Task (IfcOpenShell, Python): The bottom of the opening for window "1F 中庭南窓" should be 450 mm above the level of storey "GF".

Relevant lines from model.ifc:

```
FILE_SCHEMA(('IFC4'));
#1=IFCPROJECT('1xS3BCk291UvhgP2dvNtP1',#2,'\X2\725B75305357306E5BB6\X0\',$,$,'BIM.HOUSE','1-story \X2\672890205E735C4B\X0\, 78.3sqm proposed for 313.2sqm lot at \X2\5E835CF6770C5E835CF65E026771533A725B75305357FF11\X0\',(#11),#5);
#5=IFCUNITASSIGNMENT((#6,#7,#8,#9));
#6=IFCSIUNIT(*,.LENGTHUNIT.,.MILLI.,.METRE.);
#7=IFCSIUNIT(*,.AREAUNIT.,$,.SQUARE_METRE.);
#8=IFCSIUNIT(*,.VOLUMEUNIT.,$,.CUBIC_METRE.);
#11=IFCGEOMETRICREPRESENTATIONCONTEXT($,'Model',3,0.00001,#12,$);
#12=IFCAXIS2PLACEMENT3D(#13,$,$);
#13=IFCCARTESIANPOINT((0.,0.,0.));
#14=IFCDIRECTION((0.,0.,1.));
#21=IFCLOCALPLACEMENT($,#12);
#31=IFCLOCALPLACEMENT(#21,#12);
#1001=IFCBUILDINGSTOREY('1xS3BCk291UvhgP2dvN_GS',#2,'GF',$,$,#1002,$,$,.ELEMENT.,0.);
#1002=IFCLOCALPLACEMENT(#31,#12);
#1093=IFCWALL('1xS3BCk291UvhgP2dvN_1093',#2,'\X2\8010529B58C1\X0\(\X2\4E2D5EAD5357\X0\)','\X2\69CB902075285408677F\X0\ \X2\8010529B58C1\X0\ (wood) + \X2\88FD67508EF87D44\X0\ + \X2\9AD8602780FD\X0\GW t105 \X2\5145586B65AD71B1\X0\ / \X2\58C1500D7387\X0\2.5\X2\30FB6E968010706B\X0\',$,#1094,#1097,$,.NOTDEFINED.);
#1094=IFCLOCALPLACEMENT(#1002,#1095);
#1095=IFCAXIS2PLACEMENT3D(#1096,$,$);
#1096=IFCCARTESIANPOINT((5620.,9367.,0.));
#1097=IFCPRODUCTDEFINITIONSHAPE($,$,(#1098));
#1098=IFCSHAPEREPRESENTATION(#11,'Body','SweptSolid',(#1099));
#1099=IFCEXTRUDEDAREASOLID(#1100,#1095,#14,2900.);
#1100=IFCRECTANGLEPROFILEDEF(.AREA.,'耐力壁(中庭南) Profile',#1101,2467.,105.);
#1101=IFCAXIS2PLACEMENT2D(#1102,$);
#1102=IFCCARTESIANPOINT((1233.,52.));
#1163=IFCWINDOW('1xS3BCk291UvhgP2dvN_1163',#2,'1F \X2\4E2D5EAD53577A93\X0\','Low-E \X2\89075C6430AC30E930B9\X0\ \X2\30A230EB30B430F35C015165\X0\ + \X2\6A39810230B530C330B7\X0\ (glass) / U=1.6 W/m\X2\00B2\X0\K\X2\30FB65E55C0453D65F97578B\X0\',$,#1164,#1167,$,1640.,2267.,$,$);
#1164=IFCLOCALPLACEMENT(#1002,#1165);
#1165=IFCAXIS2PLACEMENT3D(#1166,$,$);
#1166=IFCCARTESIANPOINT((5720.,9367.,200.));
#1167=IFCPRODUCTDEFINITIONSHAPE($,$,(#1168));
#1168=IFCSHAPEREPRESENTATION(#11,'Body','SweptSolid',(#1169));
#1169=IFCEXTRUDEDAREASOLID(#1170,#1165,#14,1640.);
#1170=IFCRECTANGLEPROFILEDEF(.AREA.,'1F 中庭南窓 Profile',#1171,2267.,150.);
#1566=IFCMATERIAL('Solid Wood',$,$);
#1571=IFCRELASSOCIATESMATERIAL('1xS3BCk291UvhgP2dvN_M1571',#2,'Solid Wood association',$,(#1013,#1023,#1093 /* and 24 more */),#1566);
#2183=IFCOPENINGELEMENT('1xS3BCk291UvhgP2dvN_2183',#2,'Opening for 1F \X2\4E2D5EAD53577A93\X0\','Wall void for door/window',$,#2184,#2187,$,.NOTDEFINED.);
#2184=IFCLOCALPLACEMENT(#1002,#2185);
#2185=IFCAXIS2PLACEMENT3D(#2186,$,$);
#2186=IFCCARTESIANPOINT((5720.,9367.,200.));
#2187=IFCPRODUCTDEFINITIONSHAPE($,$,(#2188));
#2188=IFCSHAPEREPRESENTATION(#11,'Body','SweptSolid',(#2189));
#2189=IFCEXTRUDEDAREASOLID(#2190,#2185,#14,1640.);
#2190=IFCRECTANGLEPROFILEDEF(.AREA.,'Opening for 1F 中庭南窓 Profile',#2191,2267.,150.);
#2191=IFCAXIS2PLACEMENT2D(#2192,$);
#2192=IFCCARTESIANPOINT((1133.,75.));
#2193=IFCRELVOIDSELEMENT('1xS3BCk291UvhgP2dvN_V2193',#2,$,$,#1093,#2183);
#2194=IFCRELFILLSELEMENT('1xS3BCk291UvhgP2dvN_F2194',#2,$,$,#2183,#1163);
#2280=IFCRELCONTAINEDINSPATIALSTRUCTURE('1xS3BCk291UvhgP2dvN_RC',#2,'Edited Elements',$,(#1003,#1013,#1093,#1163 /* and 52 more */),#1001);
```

```python
import numpy as np
import ifcopenshell
import ifcopenshell.api.geometry
import ifcopenshell.geom
import ifcopenshell.util.element
import ifcopenshell.util.placement
import ifcopenshell.util.shape
import ifcopenshell.util.unit

model = ifcopenshell.open("model.ifc")
unit_scale = ifcopenshell.util.unit.calculate_unit_scale(model)

window = model.by_guid("1xS3BCk291UvhgP2dvN_1163")
opening = window.FillsVoids[0].RelatingOpeningElement
storey = ifcopenshell.util.element.get_container(window, ifc_class="IfcBuildingStorey")
level = ifcopenshell.util.placement.get_local_placement(storey.ObjectPlacement)[2, 3]

# The opening's origin need not be at the sill, so measure its lowest point.
shape = ifcopenshell.geom.create_shape(ifcopenshell.geom.settings(), opening)
bottom = ifcopenshell.util.shape.get_shape_bottom_elevation(shape, shape.geometry) / unit_scale
dz = level + 0.45 / unit_scale - bottom

shift = np.array([0.0, 0.0, dz])
# The window is not placed relative to its opening, so move both.
for product in (opening, window):
    matrix = ifcopenshell.util.placement.get_local_placement(product.ObjectPlacement)
    matrix[:3, 3] += shift
    ifcopenshell.api.geometry.edit_object_placement(model, product=product, matrix=matrix, is_si=False)

print(f"moved by {dz * unit_scale:+.3f} m")

model.write("model_edited.ifc")
```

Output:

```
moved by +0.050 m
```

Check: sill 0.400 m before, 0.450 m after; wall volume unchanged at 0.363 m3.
